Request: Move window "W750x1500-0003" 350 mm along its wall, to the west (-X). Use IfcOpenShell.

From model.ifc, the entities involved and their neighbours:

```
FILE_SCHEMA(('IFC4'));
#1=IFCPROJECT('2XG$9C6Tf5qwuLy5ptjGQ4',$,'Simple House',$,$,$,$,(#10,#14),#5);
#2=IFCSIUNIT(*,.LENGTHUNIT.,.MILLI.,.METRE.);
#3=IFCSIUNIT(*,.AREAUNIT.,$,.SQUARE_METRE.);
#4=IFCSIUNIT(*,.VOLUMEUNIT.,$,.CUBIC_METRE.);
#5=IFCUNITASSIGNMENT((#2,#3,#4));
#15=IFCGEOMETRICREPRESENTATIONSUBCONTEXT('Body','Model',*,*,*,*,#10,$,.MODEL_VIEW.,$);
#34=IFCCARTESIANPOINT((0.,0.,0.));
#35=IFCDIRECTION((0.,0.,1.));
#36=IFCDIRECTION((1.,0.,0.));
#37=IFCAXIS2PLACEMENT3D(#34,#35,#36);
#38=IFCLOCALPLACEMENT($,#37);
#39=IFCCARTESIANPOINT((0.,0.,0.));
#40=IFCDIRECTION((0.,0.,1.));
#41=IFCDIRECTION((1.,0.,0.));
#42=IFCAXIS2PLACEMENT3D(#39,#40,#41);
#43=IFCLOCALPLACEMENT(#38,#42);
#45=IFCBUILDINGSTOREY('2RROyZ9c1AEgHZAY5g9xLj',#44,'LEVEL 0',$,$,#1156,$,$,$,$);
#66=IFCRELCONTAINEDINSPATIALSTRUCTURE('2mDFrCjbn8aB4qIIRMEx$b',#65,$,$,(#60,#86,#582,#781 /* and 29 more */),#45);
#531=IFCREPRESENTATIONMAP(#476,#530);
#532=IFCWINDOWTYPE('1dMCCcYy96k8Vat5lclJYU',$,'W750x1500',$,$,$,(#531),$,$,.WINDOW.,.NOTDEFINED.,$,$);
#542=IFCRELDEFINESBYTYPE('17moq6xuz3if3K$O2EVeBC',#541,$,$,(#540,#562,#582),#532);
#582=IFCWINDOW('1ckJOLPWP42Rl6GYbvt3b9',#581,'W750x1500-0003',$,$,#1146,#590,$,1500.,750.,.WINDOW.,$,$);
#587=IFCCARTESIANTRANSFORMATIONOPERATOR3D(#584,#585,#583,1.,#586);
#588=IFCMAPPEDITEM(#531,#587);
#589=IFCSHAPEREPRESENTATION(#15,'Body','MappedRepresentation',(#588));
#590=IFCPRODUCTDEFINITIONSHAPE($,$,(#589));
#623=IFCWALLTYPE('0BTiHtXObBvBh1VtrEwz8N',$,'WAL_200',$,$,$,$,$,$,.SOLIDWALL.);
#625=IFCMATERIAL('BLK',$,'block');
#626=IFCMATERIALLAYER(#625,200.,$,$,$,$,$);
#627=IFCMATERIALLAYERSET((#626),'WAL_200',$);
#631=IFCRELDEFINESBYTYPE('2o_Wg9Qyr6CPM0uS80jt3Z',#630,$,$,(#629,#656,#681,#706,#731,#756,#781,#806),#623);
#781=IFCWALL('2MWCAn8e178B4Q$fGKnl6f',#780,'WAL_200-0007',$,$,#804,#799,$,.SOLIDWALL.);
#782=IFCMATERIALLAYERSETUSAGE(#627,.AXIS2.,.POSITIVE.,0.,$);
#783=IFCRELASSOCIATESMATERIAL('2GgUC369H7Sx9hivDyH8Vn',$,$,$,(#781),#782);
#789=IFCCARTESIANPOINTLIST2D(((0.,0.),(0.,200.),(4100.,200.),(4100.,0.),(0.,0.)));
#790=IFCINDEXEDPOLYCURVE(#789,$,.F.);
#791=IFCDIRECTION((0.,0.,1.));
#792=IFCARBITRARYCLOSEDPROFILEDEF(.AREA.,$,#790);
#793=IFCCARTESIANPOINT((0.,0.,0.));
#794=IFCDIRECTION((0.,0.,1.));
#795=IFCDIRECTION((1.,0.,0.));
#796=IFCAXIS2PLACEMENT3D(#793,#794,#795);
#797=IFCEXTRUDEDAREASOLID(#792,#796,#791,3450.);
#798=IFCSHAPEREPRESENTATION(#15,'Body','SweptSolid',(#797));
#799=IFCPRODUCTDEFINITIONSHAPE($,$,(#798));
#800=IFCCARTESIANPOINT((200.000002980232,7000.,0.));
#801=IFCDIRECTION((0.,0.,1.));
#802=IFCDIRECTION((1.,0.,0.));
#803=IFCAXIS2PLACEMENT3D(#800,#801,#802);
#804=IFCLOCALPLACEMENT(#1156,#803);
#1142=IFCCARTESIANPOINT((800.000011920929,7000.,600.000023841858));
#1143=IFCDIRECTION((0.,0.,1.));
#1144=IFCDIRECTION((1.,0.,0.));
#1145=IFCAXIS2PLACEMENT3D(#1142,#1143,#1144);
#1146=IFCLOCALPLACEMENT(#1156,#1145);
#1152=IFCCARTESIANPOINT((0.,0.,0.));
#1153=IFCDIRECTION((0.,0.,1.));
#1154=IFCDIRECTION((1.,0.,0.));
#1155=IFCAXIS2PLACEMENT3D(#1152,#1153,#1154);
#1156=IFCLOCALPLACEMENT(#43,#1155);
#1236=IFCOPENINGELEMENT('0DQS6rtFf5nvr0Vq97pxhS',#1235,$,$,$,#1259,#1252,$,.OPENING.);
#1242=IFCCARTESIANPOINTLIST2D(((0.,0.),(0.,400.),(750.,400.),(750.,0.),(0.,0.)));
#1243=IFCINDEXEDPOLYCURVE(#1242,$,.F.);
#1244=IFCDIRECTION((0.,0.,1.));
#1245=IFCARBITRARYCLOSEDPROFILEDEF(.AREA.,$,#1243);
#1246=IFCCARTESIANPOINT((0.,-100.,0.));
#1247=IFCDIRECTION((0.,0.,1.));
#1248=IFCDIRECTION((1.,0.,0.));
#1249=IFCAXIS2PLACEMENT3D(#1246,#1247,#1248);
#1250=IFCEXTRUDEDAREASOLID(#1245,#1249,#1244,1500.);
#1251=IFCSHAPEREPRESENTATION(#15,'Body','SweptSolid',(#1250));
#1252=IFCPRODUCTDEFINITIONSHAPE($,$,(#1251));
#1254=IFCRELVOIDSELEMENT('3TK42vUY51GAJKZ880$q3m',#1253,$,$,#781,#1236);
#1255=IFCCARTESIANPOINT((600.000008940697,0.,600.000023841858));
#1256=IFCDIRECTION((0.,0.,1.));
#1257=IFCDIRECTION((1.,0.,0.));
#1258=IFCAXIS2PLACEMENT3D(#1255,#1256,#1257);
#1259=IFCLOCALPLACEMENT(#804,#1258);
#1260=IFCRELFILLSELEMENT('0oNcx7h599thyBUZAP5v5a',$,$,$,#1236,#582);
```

```python
import ifcopenshell
import ifcopenshell.api.geometry
import ifcopenshell.util.placement

model = ifcopenshell.open("model.ifc")

window = model.by_guid("1ckJOLPWP42Rl6GYbvt3b9")
opening = window.FillsVoids[0].RelatingOpeningElement
wall = opening.VoidsElements[0].RelatingBuildingElement

wall_matrix = ifcopenshell.util.placement.get_local_placement(wall.ObjectPlacement)
shift = wall_matrix[:3, 0] * -350.0
before = ifcopenshell.util.placement.get_local_placement(window.ObjectPlacement)[:3, 3].copy()

# The window is not placed relative to its opening, so move both.
for product in (opening, window):
    matrix = ifcopenshell.util.placement.get_local_placement(product.ObjectPlacement)
    matrix[:3, 3] += shift
    ifcopenshell.api.geometry.edit_object_placement(model, product=product, matrix=matrix, is_si=False)

after = ifcopenshell.util.placement.get_local_placement(window.ObjectPlacement)[:3, 3]
print("window moved by", (after - before).round(3) + 0.0)

model.write("model_updated.ifc")
```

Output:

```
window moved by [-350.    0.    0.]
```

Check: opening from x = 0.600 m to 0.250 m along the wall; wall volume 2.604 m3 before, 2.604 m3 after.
